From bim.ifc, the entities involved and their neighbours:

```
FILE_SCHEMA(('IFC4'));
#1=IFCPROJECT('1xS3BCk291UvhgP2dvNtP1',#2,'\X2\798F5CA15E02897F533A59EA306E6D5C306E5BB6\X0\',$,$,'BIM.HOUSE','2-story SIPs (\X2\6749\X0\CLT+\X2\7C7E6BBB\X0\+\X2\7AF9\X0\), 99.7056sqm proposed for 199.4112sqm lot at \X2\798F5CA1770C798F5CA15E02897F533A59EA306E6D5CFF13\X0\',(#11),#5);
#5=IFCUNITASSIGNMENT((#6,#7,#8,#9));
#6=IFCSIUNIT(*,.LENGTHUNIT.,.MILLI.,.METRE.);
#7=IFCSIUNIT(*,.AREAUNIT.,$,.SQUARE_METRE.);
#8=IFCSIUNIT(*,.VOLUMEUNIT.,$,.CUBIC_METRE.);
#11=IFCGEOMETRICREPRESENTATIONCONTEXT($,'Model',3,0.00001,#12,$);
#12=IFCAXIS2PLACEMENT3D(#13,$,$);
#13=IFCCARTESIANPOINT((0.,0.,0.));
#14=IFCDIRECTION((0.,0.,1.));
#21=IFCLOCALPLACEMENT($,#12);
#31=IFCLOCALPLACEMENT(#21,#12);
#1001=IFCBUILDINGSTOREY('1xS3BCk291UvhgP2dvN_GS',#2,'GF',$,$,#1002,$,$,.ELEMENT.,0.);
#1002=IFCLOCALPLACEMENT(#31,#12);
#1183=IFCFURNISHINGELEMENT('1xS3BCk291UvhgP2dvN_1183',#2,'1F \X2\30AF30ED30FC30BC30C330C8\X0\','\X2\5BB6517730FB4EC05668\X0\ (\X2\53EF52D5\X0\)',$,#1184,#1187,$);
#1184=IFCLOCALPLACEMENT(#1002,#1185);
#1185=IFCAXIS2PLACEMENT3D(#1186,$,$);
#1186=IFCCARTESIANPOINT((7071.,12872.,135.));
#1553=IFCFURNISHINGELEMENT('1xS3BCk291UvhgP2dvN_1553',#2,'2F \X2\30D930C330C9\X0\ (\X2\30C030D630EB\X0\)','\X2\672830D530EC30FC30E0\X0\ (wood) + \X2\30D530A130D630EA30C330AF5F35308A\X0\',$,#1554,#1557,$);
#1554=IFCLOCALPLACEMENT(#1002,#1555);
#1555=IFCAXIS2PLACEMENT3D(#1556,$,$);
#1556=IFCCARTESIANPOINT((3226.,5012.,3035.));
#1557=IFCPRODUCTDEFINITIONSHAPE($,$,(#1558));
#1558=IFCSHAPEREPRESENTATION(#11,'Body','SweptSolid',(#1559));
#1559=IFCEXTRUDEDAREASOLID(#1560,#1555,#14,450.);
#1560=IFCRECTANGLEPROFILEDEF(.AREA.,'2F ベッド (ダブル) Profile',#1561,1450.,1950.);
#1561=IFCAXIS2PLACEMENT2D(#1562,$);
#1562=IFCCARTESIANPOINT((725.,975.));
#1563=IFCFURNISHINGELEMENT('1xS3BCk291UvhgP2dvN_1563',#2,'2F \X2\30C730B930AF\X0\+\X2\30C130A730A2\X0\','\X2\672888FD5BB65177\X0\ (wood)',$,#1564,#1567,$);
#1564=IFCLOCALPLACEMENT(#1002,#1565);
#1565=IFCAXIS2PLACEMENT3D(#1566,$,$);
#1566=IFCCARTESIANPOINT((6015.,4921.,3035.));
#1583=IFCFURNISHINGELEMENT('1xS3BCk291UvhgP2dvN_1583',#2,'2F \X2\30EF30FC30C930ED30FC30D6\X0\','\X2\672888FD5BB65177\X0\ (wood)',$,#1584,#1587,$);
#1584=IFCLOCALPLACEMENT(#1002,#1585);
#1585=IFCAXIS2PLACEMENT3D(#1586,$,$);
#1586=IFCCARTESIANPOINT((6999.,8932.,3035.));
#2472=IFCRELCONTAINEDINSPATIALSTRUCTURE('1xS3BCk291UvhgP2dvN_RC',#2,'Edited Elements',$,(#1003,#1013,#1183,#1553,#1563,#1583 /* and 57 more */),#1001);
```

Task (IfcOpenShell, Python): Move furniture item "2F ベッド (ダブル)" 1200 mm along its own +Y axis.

```python
import ifcopenshell
import ifcopenshell.api.geometry
import ifcopenshell.util.placement
import ifcopenshell.util.unit

model = ifcopenshell.open("bim.ifc")
unit_scale = ifcopenshell.util.unit.calculate_unit_scale(model)

item = model.by_id(1553)
matrix = ifcopenshell.util.placement.get_local_placement(item.ObjectPlacement)
matrix[:3, 3] += matrix[:3, 1] * 1.2 / unit_scale
ifcopenshell.api.geometry.edit_object_placement(model, product=item, matrix=matrix, is_si=False)

print(ifcopenshell.util.placement.get_local_placement(item.ObjectPlacement).round(3) + 0.0)

model.write("bim-out.ifc")
```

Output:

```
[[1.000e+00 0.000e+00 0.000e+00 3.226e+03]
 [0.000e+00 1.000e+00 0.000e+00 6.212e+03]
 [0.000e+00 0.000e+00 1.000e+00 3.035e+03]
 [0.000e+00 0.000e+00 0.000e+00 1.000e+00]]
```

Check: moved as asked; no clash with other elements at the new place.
